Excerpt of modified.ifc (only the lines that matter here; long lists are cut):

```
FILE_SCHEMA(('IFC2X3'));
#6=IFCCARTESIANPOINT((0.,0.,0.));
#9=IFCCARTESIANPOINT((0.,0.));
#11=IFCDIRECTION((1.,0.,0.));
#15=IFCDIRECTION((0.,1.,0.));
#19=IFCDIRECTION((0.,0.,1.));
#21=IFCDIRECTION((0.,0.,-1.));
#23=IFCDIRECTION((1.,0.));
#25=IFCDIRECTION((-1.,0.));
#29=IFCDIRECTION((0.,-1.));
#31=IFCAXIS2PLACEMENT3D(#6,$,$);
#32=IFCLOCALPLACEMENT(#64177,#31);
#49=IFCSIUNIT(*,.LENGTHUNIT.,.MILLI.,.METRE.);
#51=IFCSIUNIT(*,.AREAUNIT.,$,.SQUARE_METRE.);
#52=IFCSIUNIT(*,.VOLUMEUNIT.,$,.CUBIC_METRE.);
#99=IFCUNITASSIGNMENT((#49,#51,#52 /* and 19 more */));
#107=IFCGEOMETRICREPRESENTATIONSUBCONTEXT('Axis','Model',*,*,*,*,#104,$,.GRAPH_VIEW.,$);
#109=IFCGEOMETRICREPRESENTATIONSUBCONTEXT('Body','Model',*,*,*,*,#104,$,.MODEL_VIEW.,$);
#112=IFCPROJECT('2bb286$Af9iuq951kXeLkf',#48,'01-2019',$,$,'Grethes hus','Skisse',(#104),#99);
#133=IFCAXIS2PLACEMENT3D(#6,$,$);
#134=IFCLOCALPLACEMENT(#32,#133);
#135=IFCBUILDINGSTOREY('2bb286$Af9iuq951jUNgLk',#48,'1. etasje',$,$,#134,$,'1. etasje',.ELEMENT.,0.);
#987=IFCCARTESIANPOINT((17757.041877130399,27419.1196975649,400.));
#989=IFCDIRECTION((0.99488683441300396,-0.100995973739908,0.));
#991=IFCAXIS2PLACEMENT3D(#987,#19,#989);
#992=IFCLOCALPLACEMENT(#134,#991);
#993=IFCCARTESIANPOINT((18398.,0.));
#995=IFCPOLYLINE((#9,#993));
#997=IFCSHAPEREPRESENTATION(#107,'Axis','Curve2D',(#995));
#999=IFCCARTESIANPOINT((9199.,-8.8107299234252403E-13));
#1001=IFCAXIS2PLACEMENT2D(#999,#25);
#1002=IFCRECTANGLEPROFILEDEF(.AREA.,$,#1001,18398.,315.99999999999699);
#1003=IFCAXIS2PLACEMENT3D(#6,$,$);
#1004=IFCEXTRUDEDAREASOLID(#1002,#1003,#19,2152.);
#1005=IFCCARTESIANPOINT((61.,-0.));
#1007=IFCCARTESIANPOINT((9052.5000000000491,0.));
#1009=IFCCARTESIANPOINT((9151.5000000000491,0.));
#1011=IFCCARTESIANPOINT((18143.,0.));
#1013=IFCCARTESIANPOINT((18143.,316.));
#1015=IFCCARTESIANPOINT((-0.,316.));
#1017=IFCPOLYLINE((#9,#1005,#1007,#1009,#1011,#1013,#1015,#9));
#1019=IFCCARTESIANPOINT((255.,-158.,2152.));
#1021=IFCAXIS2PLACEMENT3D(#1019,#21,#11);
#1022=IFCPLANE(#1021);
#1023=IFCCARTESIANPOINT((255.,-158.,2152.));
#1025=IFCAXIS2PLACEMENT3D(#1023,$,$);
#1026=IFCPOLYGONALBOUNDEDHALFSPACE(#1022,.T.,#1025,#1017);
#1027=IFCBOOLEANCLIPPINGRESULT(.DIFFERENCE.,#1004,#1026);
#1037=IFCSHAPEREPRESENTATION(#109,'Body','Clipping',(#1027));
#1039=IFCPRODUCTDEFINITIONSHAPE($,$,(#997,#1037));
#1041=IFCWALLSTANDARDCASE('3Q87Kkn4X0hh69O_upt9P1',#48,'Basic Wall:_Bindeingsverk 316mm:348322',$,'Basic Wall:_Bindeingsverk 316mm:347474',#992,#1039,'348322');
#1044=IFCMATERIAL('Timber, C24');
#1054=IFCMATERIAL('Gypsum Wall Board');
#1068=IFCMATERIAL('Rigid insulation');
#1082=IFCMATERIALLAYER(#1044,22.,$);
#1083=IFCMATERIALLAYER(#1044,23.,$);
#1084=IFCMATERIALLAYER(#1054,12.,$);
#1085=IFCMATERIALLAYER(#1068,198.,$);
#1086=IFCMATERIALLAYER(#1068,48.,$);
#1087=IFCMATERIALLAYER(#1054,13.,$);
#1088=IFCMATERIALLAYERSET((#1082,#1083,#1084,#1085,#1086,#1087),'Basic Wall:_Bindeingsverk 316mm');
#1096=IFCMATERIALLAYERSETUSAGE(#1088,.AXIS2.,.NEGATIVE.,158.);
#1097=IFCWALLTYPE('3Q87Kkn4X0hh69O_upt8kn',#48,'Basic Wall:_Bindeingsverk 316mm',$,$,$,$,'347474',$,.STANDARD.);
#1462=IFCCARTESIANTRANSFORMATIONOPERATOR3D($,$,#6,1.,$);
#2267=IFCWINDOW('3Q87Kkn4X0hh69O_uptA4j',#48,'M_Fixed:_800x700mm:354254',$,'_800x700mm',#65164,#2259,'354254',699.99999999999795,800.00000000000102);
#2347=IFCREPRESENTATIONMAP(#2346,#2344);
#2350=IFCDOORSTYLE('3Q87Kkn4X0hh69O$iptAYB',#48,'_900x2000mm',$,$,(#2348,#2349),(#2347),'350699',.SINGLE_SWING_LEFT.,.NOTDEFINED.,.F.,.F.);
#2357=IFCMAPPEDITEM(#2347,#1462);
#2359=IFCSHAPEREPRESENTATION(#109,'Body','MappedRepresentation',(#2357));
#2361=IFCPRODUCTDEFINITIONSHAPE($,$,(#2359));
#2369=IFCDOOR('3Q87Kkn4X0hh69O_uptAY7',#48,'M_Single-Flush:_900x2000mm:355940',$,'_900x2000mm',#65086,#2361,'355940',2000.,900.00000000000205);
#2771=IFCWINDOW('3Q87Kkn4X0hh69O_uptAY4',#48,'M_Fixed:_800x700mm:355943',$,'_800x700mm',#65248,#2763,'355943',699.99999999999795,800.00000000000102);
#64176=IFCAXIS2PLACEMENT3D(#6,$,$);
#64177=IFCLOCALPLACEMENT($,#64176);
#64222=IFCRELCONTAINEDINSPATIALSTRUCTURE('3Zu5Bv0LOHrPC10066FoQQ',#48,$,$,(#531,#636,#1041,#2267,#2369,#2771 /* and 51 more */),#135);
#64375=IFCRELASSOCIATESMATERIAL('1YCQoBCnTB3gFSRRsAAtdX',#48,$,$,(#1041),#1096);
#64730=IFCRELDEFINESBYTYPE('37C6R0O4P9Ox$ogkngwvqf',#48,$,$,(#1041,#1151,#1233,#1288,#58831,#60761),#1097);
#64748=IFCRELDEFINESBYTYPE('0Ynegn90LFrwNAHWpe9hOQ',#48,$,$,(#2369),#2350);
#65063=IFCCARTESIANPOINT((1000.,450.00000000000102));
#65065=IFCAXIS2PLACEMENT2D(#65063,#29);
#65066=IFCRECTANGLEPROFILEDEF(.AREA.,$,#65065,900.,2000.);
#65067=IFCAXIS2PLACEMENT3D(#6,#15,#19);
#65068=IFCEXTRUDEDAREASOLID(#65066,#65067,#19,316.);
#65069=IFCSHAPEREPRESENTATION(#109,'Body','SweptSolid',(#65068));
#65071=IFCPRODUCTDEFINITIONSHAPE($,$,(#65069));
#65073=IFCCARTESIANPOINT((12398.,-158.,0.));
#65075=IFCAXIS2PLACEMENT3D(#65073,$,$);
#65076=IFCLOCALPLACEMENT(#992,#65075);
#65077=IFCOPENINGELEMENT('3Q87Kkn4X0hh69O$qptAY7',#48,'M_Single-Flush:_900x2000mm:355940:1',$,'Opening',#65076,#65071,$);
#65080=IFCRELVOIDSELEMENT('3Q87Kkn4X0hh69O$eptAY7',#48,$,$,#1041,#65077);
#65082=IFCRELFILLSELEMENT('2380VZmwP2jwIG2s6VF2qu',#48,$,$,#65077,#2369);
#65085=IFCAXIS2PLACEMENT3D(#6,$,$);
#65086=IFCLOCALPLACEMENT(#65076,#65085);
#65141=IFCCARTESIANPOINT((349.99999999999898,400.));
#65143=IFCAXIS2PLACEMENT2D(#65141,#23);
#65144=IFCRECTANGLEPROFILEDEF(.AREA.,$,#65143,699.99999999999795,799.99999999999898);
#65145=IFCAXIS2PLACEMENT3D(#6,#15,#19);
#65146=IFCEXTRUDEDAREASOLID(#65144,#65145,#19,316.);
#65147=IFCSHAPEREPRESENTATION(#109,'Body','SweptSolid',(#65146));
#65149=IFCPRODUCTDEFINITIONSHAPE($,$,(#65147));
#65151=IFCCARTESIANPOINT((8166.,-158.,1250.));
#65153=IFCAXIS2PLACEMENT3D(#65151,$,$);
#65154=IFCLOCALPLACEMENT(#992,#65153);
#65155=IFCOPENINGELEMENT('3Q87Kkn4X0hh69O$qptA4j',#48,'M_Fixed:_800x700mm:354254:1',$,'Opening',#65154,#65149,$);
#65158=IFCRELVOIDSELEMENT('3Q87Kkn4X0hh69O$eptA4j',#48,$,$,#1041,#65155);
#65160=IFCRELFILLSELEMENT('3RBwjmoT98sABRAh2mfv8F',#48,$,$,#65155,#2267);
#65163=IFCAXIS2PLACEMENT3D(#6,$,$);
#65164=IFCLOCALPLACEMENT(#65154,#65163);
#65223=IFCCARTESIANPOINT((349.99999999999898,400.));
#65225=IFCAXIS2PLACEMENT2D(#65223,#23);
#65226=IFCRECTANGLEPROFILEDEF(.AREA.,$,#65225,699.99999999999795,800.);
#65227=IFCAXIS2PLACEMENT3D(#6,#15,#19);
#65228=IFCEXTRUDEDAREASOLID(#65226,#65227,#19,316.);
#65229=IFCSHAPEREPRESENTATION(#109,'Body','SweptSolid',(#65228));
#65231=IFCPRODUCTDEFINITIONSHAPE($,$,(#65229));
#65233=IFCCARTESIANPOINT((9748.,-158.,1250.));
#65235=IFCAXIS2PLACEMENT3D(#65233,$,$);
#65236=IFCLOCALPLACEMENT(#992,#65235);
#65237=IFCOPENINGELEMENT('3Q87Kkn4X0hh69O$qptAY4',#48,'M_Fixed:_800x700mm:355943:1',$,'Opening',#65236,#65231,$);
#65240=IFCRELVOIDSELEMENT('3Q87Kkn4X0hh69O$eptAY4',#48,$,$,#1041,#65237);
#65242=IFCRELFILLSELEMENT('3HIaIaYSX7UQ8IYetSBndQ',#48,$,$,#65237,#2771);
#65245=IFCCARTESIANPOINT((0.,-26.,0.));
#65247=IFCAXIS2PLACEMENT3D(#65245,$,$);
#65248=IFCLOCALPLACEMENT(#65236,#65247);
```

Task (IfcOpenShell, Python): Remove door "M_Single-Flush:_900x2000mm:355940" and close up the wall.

```python
import ifcopenshell
import ifcopenshell.api.feature
import ifcopenshell.api.root
import ifcopenshell.geom
import ifcopenshell.util.shape

model = ifcopenshell.open("modified.ifc")
settings = ifcopenshell.geom.settings()


def volume(element):
    """Net volume in cubic metres, openings subtracted."""
    shape = ifcopenshell.geom.create_shape(settings, element)
    return ifcopenshell.util.shape.get_volume(shape.geometry)


door = model.by_guid("3Q87Kkn4X0hh69O_uptAY7")
opening = door.FillsVoids[0].RelatingOpeningElement
wall = opening.VoidsElements[0].RelatingBuildingElement
before = volume(wall)

ifcopenshell.api.root.remove_product(model, product=door)
ifcopenshell.api.feature.remove_feature(model, feature=opening)

after = volume(wall)

print(f"wall volume {before:.3f} -> {after:.3f} m3")

model.write("modified_rev.ifc")
```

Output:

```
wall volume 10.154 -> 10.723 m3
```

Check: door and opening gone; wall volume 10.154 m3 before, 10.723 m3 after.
